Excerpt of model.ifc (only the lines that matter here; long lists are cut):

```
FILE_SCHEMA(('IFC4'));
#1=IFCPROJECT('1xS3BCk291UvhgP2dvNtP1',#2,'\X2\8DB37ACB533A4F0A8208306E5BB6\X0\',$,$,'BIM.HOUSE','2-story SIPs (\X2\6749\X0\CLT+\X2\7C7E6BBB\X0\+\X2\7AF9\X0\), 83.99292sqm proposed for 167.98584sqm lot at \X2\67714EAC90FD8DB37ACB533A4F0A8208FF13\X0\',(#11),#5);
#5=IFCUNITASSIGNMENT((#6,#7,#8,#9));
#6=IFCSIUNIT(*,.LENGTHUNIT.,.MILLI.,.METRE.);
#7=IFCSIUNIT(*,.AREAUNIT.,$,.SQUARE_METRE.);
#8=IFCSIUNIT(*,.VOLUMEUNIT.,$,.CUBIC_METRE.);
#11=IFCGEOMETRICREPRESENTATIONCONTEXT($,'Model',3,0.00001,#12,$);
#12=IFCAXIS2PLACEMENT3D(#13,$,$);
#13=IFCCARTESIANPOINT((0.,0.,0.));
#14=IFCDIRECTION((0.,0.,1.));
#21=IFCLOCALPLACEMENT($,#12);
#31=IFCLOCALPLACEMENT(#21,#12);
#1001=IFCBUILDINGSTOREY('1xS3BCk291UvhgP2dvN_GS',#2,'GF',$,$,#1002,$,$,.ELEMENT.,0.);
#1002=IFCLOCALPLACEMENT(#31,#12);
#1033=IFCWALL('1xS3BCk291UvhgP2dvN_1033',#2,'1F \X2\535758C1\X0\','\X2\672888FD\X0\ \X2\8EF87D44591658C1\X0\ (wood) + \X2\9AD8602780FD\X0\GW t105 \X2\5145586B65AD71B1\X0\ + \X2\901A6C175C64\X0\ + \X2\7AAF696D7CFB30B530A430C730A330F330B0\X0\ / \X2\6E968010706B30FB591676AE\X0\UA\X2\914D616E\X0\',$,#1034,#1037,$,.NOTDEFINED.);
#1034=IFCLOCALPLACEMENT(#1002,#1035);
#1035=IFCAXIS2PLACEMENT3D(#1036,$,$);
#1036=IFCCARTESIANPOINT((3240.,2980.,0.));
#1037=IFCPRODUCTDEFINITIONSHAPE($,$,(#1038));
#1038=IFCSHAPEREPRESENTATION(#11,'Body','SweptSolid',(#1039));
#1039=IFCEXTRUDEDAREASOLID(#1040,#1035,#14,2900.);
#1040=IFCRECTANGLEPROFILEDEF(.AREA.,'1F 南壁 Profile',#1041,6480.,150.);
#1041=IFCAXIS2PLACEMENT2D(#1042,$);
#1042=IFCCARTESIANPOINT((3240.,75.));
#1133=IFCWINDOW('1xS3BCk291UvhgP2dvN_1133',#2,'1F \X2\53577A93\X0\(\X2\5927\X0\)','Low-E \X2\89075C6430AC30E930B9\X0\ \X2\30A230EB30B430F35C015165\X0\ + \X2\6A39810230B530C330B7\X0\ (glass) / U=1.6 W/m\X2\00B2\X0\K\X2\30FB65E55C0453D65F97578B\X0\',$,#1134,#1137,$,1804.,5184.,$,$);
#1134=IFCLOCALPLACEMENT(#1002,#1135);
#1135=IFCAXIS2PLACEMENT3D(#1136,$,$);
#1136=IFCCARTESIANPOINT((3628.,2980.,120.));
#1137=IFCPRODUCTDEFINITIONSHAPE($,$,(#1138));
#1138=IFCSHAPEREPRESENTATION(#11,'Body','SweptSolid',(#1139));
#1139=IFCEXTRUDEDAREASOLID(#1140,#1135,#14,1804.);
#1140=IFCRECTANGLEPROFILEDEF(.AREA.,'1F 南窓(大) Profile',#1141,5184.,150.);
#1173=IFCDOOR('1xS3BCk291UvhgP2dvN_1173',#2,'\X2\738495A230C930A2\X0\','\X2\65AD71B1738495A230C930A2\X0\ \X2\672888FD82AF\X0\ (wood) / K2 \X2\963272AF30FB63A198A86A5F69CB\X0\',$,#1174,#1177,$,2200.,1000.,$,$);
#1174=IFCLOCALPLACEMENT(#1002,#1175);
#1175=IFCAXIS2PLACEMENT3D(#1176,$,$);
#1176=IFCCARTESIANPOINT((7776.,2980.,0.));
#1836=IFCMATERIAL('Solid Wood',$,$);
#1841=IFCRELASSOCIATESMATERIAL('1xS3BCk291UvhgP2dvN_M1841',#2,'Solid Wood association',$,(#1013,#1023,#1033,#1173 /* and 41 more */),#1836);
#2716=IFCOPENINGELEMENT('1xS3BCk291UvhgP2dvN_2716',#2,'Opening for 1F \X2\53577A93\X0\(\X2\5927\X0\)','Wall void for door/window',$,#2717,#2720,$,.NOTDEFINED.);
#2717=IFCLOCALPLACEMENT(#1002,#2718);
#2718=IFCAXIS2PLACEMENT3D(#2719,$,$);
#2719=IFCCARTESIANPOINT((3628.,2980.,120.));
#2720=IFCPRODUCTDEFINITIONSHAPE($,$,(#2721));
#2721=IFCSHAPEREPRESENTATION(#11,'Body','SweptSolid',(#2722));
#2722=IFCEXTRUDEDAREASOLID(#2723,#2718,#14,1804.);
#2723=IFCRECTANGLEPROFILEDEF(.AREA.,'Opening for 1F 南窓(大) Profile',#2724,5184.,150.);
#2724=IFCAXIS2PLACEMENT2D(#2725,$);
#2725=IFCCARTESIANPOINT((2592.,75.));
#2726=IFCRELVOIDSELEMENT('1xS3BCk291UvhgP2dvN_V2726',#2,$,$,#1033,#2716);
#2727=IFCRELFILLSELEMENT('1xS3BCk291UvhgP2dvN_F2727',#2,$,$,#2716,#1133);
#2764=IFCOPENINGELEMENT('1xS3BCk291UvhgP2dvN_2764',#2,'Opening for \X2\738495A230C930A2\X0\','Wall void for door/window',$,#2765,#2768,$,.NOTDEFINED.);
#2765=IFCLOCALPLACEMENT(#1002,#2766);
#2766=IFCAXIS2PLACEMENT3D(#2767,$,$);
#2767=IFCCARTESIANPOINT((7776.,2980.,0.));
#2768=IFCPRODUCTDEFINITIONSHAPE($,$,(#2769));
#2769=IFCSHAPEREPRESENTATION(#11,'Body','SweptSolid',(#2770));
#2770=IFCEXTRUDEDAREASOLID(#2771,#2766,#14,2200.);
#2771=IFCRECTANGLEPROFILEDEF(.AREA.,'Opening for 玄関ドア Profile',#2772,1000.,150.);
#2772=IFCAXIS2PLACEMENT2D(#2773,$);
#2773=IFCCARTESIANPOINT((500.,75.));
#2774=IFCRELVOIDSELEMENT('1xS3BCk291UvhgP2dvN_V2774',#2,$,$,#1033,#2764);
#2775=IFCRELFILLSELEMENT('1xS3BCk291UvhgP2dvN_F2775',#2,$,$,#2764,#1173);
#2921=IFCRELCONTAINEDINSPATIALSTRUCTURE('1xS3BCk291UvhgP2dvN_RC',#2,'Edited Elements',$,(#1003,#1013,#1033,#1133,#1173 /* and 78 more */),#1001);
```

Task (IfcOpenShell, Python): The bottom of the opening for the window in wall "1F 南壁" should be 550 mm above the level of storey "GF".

```python
import numpy as np
import ifcopenshell
import ifcopenshell.api.geometry
import ifcopenshell.geom
import ifcopenshell.util.element
import ifcopenshell.util.placement
import ifcopenshell.util.shape
import ifcopenshell.util.unit

model = ifcopenshell.open("model.ifc")
unit_scale = ifcopenshell.util.unit.calculate_unit_scale(model)

window = model.by_id(1133)
opening = window.FillsVoids[0].RelatingOpeningElement
storey = ifcopenshell.util.element.get_container(window, ifc_class="IfcBuildingStorey")
level = ifcopenshell.util.placement.get_local_placement(storey.ObjectPlacement)[2, 3]

# The opening's origin need not be at the sill, so measure its lowest point.
shape = ifcopenshell.geom.create_shape(ifcopenshell.geom.settings(), opening)
bottom = ifcopenshell.util.shape.get_shape_bottom_elevation(shape, shape.geometry) / unit_scale
dz = level + 550.0 - bottom

shift = np.array([0.0, 0.0, dz])
# The window is not placed relative to its opening, so move both.
for product in (opening, window):
    matrix = ifcopenshell.util.placement.get_local_placement(product.ObjectPlacement)
    matrix[:3, 3] += shift
    ifcopenshell.api.geometry.edit_object_placement(model, product=product, matrix=matrix, is_si=False)

print(f"moved by {dz * unit_scale:+.3f} m")

model.write("model-out.ifc")
```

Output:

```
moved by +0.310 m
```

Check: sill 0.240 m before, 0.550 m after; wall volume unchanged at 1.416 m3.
